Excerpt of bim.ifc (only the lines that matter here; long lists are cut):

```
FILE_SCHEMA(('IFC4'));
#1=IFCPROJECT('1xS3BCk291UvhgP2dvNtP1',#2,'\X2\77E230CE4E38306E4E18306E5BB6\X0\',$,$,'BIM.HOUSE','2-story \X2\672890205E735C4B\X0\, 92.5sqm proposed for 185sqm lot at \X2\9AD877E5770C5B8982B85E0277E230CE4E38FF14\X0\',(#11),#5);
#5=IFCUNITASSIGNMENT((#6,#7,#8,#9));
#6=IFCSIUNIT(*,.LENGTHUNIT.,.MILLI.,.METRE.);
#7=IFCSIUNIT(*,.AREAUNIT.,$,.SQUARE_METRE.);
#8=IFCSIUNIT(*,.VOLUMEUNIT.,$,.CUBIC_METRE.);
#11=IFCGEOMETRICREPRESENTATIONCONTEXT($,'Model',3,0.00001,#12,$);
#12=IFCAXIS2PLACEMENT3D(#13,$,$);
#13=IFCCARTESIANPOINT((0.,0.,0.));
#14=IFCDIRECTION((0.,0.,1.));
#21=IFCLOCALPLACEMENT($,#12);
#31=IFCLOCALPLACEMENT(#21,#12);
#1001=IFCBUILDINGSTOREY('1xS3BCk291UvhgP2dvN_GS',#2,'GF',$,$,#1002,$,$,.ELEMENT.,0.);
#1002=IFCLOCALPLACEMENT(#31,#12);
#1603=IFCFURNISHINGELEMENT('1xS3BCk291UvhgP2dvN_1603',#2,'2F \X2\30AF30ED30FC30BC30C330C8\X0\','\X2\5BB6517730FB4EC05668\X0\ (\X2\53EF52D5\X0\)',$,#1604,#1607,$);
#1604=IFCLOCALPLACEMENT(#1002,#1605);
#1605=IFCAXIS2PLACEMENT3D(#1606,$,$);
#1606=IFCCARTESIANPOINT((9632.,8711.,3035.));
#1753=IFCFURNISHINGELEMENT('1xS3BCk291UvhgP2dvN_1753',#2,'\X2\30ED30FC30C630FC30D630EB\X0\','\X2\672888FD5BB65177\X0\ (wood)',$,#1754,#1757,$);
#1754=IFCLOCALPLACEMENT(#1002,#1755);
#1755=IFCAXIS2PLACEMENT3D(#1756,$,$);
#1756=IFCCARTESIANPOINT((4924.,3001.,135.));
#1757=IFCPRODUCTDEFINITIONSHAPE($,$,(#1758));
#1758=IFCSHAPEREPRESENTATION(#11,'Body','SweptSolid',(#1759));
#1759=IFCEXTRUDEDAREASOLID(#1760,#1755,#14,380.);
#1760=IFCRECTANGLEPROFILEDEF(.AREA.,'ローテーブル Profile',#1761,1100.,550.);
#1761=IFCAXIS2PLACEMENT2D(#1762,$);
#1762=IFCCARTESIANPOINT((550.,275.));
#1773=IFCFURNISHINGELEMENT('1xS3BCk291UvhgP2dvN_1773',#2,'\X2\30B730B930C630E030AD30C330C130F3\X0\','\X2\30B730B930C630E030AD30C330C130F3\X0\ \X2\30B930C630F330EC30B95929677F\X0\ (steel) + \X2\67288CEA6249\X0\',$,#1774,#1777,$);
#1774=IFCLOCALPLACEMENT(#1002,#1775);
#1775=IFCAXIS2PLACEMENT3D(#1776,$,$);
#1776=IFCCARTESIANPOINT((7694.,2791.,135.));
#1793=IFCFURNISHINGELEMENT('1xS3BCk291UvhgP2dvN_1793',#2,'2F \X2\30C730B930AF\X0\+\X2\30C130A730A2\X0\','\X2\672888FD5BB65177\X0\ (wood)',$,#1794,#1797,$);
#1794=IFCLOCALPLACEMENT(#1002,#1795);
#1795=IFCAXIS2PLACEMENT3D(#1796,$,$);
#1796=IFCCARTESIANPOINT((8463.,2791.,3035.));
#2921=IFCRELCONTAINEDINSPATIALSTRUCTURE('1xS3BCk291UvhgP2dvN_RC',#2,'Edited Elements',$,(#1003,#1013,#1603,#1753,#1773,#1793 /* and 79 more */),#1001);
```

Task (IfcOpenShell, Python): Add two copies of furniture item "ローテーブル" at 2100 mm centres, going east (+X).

```python
import numpy as np
import ifcopenshell
import ifcopenshell.api.geometry
import ifcopenshell.api.root
import ifcopenshell.util.element
import ifcopenshell.util.placement

model = ifcopenshell.open("bim.ifc")


def reuse_history(source, copy):
    """copy_class also copies each property set's owner history, people and application; keep the originals."""
    for rel in copy.IsDefinedBy:
        if rel.is_a("IfcRelDefinesByProperties") and (history := rel.RelatingPropertyDefinition.OwnerHistory):
            rel.RelatingPropertyDefinition.OwnerHistory = source.OwnerHistory
            ifcopenshell.util.element.remove_deep2(model, history)


source = model.by_guid("1xS3BCk291UvhgP2dvN_1753")
base = ifcopenshell.util.placement.get_local_placement(source.ObjectPlacement)
step = np.array([1.0, 0.0, 0.0]) * 2100.0

for i in range(1, 3):
    copy = ifcopenshell.api.root.copy_class(model, product=source)
    copy.Representation = ifcopenshell.util.element.copy_deep(
        model, source.Representation, exclude=["IfcGeometricRepresentationContext", "IfcRepresentationMap"]
    )
    reuse_history(source, copy)
    matrix = base.copy()
    matrix[:3, 3] += i * step
    print("added at", matrix[:3, 3].round(3) + 0.0)
    ifcopenshell.api.geometry.edit_object_placement(model, product=copy, matrix=matrix, is_si=False)

model.write("bim_edited.ifc")
```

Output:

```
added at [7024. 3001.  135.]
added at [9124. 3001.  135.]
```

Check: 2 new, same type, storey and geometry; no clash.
